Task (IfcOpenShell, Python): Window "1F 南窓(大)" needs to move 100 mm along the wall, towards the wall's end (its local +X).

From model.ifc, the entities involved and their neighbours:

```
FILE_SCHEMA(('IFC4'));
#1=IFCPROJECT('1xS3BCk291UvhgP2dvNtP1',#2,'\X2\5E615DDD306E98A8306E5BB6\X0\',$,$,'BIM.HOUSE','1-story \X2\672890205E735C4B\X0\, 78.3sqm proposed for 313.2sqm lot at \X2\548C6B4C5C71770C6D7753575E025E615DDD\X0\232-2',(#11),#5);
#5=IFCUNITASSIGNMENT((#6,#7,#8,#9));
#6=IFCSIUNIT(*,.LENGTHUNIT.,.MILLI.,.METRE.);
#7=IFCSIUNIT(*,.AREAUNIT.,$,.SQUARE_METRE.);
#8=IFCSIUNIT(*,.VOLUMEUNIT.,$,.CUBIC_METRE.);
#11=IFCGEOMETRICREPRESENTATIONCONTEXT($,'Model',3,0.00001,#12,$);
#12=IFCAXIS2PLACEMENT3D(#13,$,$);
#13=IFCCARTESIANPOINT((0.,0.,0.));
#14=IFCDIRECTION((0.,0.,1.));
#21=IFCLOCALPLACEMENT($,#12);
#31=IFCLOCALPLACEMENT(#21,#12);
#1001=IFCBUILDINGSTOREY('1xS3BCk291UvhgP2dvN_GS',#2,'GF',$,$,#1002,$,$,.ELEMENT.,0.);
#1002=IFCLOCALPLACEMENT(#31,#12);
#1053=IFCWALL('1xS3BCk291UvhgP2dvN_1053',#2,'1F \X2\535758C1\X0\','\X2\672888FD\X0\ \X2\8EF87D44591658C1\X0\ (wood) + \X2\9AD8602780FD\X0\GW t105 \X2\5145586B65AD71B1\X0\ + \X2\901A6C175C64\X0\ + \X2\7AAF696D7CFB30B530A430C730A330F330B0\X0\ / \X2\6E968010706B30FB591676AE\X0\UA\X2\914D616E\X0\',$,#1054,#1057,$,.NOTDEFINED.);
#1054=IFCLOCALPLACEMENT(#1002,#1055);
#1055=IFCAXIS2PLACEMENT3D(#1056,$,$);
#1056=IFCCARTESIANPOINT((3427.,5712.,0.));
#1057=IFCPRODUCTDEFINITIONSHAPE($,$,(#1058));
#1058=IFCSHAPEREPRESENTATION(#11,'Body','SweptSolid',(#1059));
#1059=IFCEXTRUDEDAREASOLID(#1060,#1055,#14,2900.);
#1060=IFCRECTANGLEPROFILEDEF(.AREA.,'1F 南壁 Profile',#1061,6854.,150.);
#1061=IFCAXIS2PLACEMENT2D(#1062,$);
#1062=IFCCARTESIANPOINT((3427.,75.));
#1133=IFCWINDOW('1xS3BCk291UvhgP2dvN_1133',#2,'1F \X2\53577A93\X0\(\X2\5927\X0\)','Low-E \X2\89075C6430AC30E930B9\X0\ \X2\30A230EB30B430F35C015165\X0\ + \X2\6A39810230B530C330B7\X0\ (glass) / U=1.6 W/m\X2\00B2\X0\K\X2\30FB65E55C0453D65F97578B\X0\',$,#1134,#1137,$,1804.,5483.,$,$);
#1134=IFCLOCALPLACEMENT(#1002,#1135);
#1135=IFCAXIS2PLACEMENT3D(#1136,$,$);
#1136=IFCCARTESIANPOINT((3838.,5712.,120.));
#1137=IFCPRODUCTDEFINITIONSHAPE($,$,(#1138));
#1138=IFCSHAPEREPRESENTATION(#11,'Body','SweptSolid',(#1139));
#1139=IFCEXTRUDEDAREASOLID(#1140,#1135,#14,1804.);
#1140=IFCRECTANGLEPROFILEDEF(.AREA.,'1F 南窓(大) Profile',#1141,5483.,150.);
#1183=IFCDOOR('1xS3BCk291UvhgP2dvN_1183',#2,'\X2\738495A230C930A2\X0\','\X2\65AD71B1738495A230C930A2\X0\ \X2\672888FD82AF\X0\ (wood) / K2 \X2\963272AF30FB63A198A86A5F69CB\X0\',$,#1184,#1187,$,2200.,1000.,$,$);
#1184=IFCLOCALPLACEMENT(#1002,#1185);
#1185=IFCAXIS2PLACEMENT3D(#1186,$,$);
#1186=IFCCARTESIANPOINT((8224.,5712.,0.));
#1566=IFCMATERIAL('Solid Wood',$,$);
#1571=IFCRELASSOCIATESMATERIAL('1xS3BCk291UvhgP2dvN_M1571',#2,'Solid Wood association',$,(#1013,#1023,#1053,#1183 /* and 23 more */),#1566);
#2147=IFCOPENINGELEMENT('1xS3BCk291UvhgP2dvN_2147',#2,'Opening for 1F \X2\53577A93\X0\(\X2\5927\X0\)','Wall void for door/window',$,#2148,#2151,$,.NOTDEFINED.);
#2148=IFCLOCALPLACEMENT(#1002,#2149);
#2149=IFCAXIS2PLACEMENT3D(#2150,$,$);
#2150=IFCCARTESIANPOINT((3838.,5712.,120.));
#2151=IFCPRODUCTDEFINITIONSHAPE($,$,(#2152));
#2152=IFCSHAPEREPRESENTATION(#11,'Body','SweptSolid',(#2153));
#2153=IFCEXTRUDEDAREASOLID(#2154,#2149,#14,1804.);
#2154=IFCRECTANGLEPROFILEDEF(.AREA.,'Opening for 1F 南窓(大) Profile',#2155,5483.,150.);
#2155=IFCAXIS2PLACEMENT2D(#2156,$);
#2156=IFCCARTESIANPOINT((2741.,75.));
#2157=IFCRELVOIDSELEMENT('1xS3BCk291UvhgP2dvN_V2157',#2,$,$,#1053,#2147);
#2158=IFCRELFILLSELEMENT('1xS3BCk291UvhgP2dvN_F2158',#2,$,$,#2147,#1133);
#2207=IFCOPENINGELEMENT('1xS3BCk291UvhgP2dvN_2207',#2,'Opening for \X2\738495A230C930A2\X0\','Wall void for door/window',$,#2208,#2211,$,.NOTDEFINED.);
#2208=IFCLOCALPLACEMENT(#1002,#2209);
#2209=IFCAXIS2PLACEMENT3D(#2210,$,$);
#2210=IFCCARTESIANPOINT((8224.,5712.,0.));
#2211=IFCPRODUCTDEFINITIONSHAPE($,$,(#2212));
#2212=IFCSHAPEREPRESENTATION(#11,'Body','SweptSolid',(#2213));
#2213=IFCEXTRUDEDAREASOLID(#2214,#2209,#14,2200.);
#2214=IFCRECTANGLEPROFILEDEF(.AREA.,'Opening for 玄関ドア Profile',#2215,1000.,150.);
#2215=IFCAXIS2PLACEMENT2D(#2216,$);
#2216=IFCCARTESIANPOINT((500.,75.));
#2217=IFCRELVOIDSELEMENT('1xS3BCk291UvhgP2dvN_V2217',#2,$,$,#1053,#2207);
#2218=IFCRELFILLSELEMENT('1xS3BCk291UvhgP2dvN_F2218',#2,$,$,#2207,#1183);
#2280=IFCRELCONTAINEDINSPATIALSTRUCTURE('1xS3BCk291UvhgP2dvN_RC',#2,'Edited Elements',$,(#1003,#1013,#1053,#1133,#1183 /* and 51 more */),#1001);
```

```python
import ifcopenshell
import ifcopenshell.api.geometry
import ifcopenshell.util.placement

model = ifcopenshell.open("model.ifc")

window = model.by_id(1133)
opening = window.FillsVoids[0].RelatingOpeningElement
wall = opening.VoidsElements[0].RelatingBuildingElement

wall_matrix = ifcopenshell.util.placement.get_local_placement(wall.ObjectPlacement)
shift = wall_matrix[:3, 0] * 100.0
before = ifcopenshell.util.placement.get_local_placement(window.ObjectPlacement)[:3, 3].copy()

# The window is not placed relative to its opening, so move both.
for product in (opening, window):
    matrix = ifcopenshell.util.placement.get_local_placement(product.ObjectPlacement)
    matrix[:3, 3] += shift
    ifcopenshell.api.geometry.edit_object_placement(model, product=product, matrix=matrix, is_si=False)

after = ifcopenshell.util.placement.get_local_placement(window.ObjectPlacement)[:3, 3]
print("window moved by", (after - before).round(3) + 0.0)

model.write("model-out.ifc")
```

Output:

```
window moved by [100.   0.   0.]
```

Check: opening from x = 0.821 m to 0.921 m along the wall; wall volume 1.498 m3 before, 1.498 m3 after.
